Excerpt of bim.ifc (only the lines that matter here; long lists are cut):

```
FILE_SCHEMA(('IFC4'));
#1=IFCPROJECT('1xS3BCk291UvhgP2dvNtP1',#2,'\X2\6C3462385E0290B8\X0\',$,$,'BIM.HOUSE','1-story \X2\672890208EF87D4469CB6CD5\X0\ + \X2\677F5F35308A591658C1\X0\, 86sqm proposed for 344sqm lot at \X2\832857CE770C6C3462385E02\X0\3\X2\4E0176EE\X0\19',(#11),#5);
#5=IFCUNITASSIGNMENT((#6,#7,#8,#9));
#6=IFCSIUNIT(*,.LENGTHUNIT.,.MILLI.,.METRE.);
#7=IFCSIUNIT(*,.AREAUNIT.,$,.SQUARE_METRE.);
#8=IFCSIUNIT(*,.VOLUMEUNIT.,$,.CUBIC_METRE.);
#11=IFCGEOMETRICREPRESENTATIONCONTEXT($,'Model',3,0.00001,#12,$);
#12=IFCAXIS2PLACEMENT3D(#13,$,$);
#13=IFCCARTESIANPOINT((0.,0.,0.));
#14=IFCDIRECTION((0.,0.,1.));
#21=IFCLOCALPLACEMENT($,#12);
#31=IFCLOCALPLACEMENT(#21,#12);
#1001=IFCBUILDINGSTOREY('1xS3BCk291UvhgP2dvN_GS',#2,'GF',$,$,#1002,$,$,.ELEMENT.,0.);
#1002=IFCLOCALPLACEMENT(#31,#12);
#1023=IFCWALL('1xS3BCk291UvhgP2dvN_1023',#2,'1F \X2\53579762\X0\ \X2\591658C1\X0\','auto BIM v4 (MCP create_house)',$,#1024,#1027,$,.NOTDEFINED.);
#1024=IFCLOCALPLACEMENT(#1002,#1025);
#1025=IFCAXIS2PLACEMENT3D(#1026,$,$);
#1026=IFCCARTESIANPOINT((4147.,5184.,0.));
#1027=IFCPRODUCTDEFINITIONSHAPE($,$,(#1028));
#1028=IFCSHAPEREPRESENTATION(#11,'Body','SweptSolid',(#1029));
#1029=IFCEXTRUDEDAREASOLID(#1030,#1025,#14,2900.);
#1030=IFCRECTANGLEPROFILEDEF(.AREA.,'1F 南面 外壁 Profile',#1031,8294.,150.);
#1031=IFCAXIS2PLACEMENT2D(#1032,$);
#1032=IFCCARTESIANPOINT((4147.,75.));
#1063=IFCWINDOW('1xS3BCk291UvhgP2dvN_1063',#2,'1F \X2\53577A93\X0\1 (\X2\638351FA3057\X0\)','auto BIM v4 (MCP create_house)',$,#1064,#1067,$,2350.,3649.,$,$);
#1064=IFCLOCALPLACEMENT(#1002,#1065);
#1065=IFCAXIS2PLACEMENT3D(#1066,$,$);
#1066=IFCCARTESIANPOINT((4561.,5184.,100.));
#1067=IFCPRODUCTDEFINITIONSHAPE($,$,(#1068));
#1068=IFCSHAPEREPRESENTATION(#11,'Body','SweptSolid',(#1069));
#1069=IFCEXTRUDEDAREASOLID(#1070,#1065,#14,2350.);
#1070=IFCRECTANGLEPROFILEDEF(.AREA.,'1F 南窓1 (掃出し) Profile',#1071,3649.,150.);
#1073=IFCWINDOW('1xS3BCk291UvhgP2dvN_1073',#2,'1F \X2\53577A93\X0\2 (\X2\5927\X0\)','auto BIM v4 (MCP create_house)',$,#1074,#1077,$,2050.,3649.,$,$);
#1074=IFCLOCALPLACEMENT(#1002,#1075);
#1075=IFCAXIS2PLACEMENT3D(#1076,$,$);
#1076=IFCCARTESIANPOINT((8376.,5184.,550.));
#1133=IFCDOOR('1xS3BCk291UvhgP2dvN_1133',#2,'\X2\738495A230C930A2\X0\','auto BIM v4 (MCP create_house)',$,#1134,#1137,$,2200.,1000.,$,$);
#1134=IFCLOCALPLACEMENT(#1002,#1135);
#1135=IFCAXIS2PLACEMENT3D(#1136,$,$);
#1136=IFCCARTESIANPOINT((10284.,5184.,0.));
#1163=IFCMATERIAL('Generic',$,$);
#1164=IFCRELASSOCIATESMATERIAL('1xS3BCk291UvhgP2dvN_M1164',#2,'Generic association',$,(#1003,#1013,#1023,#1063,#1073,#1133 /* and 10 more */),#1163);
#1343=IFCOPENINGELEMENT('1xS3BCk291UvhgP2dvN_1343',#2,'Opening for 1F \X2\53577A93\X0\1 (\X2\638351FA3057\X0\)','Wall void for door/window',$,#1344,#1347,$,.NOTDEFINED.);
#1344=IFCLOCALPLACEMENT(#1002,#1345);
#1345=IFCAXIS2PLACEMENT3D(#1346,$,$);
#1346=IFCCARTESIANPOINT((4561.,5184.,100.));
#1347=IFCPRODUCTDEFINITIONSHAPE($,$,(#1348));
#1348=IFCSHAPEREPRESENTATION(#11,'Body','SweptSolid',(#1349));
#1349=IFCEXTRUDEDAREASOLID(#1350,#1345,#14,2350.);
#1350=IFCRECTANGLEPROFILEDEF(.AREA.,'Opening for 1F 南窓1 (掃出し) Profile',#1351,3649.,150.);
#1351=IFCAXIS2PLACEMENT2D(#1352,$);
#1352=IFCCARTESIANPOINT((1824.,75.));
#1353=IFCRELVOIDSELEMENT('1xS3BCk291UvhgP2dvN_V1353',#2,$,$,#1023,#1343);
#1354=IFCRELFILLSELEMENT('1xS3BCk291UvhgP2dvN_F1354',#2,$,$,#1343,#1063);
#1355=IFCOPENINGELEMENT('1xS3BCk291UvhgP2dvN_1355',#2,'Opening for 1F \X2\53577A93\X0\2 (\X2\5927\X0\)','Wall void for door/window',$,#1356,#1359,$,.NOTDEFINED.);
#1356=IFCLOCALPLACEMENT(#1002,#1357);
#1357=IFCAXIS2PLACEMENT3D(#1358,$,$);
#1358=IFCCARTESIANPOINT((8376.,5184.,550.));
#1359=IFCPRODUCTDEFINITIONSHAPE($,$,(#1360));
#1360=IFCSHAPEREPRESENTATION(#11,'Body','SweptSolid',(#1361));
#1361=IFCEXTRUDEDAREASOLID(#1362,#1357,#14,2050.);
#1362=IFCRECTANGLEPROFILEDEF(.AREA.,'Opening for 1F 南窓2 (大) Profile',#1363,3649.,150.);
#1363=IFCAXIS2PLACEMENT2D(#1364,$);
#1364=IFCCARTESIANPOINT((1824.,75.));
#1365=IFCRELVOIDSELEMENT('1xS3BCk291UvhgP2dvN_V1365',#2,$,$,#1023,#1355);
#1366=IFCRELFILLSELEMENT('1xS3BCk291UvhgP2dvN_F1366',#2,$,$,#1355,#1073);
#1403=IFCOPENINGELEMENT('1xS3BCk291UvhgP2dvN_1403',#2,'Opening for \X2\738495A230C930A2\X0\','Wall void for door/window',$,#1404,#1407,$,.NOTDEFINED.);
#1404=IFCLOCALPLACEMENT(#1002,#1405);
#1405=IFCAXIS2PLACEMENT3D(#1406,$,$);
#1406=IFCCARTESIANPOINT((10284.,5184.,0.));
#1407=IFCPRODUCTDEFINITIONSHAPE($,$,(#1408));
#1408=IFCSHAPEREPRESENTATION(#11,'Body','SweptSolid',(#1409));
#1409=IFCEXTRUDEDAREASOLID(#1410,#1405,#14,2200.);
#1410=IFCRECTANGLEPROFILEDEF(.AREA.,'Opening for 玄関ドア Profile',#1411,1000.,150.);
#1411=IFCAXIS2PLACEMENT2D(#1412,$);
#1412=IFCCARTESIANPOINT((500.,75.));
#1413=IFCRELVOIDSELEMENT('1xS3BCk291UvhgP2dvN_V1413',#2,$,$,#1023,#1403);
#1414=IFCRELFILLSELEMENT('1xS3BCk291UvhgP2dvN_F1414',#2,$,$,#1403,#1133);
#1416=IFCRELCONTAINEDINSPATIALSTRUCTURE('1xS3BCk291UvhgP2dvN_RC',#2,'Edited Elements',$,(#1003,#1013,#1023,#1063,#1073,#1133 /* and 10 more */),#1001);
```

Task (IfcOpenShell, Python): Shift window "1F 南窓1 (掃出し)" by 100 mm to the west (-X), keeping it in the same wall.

```python
import ifcopenshell
import ifcopenshell.api.geometry
import ifcopenshell.util.placement
import ifcopenshell.util.unit

model = ifcopenshell.open("bim.ifc")
unit_scale = ifcopenshell.util.unit.calculate_unit_scale(model)

window = model.by_guid("1xS3BCk291UvhgP2dvN_1063")
opening = window.FillsVoids[0].RelatingOpeningElement
wall = opening.VoidsElements[0].RelatingBuildingElement

wall_matrix = ifcopenshell.util.placement.get_local_placement(wall.ObjectPlacement)
shift = wall_matrix[:3, 0] * -0.1 / unit_scale
before = ifcopenshell.util.placement.get_local_placement(window.ObjectPlacement)[:3, 3].copy()

# The window is not placed relative to its opening, so move both.
for product in (opening, window):
    matrix = ifcopenshell.util.placement.get_local_placement(product.ObjectPlacement)
    matrix[:3, 3] += shift
    ifcopenshell.api.geometry.edit_object_placement(model, product=product, matrix=matrix, is_si=False)

after = ifcopenshell.util.placement.get_local_placement(window.ObjectPlacement)[:3, 3]
print("window moved by", (after - before).round(3) + 0.0)

model.write("bim_rev.ifc")
```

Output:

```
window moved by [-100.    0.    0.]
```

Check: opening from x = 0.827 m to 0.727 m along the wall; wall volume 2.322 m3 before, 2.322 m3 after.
